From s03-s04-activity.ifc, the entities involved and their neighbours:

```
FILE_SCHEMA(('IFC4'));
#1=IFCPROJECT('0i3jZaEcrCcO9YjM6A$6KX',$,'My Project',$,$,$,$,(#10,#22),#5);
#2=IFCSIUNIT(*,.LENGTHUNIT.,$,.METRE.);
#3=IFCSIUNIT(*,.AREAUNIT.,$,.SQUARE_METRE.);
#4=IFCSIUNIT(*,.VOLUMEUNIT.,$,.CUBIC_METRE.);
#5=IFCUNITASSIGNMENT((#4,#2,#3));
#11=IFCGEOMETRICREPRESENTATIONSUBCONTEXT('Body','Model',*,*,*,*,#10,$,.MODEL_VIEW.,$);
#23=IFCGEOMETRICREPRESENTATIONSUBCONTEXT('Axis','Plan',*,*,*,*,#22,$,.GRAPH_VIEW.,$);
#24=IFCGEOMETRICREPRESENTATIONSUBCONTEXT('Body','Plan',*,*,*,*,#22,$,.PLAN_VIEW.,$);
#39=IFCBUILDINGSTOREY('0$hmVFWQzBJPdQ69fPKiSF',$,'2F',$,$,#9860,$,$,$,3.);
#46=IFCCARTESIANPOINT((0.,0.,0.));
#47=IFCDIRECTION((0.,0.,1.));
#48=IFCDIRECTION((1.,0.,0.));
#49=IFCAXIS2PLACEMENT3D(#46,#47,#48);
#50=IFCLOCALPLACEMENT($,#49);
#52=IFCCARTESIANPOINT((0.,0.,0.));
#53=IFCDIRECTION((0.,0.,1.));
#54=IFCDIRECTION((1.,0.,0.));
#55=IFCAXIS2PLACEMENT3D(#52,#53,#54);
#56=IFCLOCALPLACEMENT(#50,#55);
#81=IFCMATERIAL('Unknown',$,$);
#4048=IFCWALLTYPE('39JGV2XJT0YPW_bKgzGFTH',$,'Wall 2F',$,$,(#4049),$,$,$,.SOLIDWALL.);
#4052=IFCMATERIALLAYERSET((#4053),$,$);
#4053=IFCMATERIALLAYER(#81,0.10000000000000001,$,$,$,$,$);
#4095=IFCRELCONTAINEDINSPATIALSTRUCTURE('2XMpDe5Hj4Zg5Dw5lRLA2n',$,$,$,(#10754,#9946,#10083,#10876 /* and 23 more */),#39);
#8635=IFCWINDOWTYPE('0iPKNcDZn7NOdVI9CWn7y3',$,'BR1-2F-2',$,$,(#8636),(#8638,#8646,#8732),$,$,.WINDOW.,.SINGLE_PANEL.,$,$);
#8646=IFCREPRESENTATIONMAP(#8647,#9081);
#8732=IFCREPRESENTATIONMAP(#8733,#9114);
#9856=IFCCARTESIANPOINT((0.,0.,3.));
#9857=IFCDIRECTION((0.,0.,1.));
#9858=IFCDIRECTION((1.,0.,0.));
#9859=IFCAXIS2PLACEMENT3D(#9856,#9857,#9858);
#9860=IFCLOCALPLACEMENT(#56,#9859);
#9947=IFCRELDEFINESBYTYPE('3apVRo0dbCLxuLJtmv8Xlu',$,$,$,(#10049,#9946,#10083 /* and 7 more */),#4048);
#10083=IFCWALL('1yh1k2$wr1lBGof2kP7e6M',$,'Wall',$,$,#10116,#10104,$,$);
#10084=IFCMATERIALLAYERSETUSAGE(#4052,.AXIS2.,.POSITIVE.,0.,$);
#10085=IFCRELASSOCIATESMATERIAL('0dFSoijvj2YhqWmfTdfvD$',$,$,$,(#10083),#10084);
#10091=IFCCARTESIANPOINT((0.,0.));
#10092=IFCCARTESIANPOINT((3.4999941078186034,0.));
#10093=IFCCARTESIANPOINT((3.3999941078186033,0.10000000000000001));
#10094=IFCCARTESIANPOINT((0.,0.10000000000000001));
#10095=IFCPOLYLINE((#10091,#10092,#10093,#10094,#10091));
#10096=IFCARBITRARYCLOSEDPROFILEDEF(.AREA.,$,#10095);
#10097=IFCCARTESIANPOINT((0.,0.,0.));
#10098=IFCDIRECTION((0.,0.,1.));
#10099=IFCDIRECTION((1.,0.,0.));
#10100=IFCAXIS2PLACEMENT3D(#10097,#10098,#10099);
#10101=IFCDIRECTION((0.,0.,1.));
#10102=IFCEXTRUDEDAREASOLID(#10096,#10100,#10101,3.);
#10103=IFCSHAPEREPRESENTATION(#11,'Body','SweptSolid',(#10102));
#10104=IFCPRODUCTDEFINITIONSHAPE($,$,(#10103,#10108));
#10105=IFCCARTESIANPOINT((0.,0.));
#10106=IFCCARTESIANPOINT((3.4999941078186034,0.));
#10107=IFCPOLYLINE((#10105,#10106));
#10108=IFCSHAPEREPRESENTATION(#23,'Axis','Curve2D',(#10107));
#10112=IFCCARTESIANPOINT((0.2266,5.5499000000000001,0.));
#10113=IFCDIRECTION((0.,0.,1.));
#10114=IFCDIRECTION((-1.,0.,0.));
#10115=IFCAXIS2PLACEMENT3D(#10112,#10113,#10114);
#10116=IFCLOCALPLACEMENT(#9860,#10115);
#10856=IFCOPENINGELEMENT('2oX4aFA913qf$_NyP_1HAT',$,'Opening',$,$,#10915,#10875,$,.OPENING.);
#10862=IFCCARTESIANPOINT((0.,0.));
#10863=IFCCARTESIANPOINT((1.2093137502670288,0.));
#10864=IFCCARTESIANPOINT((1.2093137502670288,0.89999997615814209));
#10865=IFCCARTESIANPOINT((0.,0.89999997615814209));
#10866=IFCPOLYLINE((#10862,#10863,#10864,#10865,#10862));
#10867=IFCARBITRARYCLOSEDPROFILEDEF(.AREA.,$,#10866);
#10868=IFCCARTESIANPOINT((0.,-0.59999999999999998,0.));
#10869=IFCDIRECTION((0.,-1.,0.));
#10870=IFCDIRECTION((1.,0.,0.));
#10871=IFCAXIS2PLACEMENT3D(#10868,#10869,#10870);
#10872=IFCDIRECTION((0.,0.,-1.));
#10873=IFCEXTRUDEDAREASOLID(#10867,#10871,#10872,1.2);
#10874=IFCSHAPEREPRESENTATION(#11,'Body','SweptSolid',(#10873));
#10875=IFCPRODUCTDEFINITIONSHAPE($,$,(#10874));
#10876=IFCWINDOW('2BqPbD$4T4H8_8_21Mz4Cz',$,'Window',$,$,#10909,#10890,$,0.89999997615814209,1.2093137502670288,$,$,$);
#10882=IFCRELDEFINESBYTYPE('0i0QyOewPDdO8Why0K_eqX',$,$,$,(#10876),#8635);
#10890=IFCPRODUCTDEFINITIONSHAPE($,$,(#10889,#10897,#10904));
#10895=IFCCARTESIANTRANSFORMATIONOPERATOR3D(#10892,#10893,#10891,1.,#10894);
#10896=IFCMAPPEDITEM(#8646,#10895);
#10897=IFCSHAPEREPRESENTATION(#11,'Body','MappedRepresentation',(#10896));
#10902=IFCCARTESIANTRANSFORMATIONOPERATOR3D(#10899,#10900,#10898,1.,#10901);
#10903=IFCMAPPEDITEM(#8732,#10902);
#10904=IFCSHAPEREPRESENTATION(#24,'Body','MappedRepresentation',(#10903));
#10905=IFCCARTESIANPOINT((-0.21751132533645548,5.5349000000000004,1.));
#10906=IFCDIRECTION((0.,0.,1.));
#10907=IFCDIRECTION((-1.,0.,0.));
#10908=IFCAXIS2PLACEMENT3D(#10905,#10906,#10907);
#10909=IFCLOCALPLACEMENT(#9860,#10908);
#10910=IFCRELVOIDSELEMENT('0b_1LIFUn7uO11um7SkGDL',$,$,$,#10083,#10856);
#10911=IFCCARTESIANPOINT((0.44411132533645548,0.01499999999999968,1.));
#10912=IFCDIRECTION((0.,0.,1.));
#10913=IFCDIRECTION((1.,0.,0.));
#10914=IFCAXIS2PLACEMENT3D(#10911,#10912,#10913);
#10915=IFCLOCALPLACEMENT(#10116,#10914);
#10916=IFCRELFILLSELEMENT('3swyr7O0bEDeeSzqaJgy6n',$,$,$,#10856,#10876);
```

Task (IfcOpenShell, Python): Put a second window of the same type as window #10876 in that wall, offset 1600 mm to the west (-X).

```python
import ifcopenshell
import ifcopenshell.api.feature
import ifcopenshell.api.geometry
import ifcopenshell.api.root
import ifcopenshell.geom
import ifcopenshell.util.element
import ifcopenshell.util.placement
import ifcopenshell.util.shape
import ifcopenshell.util.unit

model = ifcopenshell.open("s03-s04-activity.ifc")
unit_scale = ifcopenshell.util.unit.calculate_unit_scale(model)
settings = ifcopenshell.geom.settings()


def volume(element):
    """Net volume in cubic metres, openings subtracted."""
    shape = ifcopenshell.geom.create_shape(settings, element)
    return ifcopenshell.util.shape.get_volume(shape.geometry)


window = model.by_guid("2BqPbD$4T4H8_8_21Mz4Cz")
opening = window.FillsVoids[0].RelatingOpeningElement
wall = opening.VoidsElements[0].RelatingBuildingElement
before = volume(wall)
shift = ifcopenshell.util.placement.get_local_placement(wall.ObjectPlacement)[:3, 0] * 1.6 / unit_scale

# copy_class copies the void relationship, type, container and properties, but no geometry.
new_opening = ifcopenshell.api.root.copy_class(model, product=opening)
new_opening.Representation = ifcopenshell.util.element.copy_deep(
    model, opening.Representation, exclude=["IfcGeometricRepresentationContext", "IfcRepresentationMap"]
)
new_window = ifcopenshell.api.root.copy_class(model, product=window)
new_window.Representation = ifcopenshell.util.element.copy_deep(
    model, window.Representation, exclude=["IfcGeometricRepresentationContext", "IfcRepresentationMap"]
)
ifcopenshell.api.feature.add_filling(model, opening=new_opening, element=new_window)

for old, new in ((opening, new_opening), (window, new_window)):
    matrix = ifcopenshell.util.placement.get_local_placement(old.ObjectPlacement)
    matrix[:3, 3] += shift
    ifcopenshell.api.geometry.edit_object_placement(model, product=new, matrix=matrix, is_si=False)

after = volume(wall)

print(f"wall volume {before:.3f} -> {after:.3f} m3")

model.write("s03-s04-activity_v2.ifc")
```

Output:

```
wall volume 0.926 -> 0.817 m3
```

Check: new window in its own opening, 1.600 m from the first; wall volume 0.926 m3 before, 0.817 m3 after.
